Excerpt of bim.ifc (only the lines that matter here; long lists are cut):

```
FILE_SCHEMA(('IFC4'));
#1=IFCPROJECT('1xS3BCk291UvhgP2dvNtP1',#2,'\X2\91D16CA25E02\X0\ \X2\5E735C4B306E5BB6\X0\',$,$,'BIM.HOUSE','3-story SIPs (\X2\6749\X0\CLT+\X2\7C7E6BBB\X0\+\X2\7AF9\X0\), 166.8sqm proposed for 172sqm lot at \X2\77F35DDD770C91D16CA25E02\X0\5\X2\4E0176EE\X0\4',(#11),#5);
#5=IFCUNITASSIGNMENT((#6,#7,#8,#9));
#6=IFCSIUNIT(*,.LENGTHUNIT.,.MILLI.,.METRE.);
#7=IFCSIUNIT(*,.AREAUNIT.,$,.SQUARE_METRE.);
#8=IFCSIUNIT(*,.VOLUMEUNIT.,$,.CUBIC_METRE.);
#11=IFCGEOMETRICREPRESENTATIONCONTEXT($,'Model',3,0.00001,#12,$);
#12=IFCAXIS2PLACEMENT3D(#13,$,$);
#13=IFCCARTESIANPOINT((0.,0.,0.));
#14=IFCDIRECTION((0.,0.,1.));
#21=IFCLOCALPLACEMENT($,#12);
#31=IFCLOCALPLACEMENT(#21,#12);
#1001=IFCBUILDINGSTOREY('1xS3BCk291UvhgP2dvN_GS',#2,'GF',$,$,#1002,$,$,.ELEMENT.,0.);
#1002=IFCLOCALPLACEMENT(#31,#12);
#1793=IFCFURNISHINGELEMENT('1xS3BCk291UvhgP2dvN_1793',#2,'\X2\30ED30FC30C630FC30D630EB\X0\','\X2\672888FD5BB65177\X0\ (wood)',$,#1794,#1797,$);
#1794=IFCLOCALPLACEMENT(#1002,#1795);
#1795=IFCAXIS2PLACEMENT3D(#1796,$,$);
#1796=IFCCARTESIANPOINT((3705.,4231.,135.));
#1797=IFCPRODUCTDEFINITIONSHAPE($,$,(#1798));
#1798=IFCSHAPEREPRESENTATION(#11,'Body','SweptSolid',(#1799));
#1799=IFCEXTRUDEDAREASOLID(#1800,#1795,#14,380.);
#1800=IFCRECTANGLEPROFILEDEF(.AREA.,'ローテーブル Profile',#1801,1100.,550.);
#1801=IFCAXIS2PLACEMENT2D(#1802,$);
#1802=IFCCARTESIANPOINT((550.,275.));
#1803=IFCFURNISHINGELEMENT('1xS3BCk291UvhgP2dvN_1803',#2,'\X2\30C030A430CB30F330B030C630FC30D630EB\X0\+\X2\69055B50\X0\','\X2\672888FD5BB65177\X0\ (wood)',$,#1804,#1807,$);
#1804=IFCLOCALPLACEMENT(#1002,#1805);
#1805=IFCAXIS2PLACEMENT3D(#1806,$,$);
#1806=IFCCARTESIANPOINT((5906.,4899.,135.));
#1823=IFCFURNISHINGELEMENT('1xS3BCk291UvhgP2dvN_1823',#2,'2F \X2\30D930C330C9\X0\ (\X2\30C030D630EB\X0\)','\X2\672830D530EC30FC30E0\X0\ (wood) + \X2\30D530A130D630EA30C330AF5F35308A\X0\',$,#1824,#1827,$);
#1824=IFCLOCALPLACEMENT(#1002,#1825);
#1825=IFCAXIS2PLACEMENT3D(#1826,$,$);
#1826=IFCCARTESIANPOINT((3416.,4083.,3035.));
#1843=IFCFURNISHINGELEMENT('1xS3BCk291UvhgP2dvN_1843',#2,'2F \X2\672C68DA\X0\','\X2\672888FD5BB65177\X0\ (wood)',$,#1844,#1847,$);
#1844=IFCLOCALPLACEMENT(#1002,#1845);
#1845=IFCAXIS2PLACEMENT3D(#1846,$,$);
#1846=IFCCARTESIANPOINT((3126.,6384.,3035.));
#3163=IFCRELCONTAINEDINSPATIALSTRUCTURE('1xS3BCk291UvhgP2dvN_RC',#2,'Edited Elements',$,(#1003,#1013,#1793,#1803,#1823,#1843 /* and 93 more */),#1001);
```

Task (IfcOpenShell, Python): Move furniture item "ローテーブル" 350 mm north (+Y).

```python
import ifcopenshell
import ifcopenshell.api.geometry
import ifcopenshell.util.placement
import ifcopenshell.util.unit

model = ifcopenshell.open("bim.ifc")
unit_scale = ifcopenshell.util.unit.calculate_unit_scale(model)

item = model.by_guid("1xS3BCk291UvhgP2dvN_1793")
matrix = ifcopenshell.util.placement.get_local_placement(item.ObjectPlacement)
matrix[1, 3] += 0.35 / unit_scale
ifcopenshell.api.geometry.edit_object_placement(model, product=item, matrix=matrix, is_si=False)

print(ifcopenshell.util.placement.get_local_placement(item.ObjectPlacement).round(3) + 0.0)

model.write("bim_rev.ifc")
```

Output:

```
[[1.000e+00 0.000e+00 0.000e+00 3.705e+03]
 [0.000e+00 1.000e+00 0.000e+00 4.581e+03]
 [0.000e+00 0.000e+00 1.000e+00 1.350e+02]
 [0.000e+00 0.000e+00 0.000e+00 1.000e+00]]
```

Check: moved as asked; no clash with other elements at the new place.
